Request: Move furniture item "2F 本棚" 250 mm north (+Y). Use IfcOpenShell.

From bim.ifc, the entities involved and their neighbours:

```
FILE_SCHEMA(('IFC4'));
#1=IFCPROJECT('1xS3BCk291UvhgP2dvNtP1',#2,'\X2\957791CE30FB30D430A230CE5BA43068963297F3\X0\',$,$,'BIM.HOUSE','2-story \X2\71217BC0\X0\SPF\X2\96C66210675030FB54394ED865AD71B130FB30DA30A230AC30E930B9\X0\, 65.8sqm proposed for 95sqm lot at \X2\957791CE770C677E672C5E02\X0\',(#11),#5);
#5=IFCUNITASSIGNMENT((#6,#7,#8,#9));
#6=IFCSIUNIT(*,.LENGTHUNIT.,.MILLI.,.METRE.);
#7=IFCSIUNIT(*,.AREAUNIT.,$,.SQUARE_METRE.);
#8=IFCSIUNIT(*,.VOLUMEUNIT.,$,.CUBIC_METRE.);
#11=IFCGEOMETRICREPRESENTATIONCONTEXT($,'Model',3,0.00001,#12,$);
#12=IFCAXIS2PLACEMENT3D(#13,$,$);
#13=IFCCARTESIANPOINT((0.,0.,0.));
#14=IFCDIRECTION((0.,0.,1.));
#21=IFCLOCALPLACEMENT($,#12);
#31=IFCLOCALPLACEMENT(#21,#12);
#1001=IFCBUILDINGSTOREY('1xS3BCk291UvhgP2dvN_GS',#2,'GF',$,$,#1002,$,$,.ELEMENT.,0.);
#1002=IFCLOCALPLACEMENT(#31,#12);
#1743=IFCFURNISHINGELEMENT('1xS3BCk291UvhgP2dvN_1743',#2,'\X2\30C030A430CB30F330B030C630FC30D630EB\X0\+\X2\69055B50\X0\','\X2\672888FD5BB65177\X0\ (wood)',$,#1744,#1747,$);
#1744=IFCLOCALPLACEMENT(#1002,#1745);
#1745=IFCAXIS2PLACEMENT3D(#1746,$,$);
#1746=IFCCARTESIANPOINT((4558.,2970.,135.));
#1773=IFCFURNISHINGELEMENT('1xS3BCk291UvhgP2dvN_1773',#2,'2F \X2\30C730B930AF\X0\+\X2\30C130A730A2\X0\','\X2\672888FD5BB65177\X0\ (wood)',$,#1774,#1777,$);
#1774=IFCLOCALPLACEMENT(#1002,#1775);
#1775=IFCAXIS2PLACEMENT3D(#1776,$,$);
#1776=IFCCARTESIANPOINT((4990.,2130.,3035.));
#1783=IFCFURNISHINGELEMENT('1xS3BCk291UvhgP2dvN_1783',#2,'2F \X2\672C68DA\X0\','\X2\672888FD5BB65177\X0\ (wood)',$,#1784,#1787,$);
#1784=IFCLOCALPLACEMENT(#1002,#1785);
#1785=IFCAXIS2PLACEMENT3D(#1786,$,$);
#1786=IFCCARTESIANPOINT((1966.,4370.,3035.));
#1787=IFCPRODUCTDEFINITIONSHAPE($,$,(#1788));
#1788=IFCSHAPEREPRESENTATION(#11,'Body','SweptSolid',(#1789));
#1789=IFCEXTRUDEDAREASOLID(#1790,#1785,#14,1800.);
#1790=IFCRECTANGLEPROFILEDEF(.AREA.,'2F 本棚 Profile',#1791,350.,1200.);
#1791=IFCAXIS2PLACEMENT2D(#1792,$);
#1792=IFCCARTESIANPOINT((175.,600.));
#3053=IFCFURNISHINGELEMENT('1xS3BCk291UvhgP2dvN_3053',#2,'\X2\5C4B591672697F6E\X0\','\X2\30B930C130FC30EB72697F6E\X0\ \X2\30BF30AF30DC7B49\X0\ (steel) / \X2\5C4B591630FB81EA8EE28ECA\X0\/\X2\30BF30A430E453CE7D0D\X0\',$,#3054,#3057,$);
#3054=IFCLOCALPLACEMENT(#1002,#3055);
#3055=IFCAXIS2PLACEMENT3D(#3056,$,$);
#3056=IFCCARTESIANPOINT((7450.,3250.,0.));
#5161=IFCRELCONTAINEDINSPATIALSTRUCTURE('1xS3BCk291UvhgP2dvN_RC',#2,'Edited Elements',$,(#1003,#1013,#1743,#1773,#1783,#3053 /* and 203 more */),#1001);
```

```python
import ifcopenshell
import ifcopenshell.api.geometry
import ifcopenshell.util.placement
import ifcopenshell.util.unit

model = ifcopenshell.open("bim.ifc")
unit_scale = ifcopenshell.util.unit.calculate_unit_scale(model)

item = model.by_id(1783)
matrix = ifcopenshell.util.placement.get_local_placement(item.ObjectPlacement)
matrix[1, 3] += 0.25 / unit_scale
ifcopenshell.api.geometry.edit_object_placement(model, product=item, matrix=matrix, is_si=False)

print(ifcopenshell.util.placement.get_local_placement(item.ObjectPlacement).round(3) + 0.0)

model.write("bim_rev.ifc")
```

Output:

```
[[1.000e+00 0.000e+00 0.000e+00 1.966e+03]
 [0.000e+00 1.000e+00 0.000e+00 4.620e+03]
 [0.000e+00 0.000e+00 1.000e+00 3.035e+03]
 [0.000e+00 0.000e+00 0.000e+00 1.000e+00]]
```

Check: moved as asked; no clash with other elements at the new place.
